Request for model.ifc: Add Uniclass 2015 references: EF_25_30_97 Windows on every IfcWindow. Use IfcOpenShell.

First a look at what the model holds.

```python
import ifcopenshell

model = ifcopenshell.open("model.ifc")
print(model.schema)
print("classifications:", [c.Name for c in model.by_type("IfcClassification")])
for ifc_class in ("IfcDoor", "IfcRoof", "IfcStair", "IfcWall", "IfcWindow"):
    print(ifc_class, len(model.by_type(ifc_class)))
```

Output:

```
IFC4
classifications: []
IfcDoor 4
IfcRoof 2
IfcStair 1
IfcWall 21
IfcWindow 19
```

```python
import ifcopenshell
import ifcopenshell.api.classification

model = ifcopenshell.open("model.ifc")

system = ifcopenshell.api.classification.add_classification(model, classification="Uniclass 2015")

codes = {
    "IfcWindow": ("EF_25_30_97", "Windows"),
}
for ifc_class, (code, name) in codes.items():
    products = model.by_type(ifc_class)
    ifcopenshell.api.classification.add_reference(
        model, products=products, classification=system, identification=code, name=name
    )
    print(code, len(products))

model.write("model_v2.ifc")
```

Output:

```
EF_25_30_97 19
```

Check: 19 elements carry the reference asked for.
